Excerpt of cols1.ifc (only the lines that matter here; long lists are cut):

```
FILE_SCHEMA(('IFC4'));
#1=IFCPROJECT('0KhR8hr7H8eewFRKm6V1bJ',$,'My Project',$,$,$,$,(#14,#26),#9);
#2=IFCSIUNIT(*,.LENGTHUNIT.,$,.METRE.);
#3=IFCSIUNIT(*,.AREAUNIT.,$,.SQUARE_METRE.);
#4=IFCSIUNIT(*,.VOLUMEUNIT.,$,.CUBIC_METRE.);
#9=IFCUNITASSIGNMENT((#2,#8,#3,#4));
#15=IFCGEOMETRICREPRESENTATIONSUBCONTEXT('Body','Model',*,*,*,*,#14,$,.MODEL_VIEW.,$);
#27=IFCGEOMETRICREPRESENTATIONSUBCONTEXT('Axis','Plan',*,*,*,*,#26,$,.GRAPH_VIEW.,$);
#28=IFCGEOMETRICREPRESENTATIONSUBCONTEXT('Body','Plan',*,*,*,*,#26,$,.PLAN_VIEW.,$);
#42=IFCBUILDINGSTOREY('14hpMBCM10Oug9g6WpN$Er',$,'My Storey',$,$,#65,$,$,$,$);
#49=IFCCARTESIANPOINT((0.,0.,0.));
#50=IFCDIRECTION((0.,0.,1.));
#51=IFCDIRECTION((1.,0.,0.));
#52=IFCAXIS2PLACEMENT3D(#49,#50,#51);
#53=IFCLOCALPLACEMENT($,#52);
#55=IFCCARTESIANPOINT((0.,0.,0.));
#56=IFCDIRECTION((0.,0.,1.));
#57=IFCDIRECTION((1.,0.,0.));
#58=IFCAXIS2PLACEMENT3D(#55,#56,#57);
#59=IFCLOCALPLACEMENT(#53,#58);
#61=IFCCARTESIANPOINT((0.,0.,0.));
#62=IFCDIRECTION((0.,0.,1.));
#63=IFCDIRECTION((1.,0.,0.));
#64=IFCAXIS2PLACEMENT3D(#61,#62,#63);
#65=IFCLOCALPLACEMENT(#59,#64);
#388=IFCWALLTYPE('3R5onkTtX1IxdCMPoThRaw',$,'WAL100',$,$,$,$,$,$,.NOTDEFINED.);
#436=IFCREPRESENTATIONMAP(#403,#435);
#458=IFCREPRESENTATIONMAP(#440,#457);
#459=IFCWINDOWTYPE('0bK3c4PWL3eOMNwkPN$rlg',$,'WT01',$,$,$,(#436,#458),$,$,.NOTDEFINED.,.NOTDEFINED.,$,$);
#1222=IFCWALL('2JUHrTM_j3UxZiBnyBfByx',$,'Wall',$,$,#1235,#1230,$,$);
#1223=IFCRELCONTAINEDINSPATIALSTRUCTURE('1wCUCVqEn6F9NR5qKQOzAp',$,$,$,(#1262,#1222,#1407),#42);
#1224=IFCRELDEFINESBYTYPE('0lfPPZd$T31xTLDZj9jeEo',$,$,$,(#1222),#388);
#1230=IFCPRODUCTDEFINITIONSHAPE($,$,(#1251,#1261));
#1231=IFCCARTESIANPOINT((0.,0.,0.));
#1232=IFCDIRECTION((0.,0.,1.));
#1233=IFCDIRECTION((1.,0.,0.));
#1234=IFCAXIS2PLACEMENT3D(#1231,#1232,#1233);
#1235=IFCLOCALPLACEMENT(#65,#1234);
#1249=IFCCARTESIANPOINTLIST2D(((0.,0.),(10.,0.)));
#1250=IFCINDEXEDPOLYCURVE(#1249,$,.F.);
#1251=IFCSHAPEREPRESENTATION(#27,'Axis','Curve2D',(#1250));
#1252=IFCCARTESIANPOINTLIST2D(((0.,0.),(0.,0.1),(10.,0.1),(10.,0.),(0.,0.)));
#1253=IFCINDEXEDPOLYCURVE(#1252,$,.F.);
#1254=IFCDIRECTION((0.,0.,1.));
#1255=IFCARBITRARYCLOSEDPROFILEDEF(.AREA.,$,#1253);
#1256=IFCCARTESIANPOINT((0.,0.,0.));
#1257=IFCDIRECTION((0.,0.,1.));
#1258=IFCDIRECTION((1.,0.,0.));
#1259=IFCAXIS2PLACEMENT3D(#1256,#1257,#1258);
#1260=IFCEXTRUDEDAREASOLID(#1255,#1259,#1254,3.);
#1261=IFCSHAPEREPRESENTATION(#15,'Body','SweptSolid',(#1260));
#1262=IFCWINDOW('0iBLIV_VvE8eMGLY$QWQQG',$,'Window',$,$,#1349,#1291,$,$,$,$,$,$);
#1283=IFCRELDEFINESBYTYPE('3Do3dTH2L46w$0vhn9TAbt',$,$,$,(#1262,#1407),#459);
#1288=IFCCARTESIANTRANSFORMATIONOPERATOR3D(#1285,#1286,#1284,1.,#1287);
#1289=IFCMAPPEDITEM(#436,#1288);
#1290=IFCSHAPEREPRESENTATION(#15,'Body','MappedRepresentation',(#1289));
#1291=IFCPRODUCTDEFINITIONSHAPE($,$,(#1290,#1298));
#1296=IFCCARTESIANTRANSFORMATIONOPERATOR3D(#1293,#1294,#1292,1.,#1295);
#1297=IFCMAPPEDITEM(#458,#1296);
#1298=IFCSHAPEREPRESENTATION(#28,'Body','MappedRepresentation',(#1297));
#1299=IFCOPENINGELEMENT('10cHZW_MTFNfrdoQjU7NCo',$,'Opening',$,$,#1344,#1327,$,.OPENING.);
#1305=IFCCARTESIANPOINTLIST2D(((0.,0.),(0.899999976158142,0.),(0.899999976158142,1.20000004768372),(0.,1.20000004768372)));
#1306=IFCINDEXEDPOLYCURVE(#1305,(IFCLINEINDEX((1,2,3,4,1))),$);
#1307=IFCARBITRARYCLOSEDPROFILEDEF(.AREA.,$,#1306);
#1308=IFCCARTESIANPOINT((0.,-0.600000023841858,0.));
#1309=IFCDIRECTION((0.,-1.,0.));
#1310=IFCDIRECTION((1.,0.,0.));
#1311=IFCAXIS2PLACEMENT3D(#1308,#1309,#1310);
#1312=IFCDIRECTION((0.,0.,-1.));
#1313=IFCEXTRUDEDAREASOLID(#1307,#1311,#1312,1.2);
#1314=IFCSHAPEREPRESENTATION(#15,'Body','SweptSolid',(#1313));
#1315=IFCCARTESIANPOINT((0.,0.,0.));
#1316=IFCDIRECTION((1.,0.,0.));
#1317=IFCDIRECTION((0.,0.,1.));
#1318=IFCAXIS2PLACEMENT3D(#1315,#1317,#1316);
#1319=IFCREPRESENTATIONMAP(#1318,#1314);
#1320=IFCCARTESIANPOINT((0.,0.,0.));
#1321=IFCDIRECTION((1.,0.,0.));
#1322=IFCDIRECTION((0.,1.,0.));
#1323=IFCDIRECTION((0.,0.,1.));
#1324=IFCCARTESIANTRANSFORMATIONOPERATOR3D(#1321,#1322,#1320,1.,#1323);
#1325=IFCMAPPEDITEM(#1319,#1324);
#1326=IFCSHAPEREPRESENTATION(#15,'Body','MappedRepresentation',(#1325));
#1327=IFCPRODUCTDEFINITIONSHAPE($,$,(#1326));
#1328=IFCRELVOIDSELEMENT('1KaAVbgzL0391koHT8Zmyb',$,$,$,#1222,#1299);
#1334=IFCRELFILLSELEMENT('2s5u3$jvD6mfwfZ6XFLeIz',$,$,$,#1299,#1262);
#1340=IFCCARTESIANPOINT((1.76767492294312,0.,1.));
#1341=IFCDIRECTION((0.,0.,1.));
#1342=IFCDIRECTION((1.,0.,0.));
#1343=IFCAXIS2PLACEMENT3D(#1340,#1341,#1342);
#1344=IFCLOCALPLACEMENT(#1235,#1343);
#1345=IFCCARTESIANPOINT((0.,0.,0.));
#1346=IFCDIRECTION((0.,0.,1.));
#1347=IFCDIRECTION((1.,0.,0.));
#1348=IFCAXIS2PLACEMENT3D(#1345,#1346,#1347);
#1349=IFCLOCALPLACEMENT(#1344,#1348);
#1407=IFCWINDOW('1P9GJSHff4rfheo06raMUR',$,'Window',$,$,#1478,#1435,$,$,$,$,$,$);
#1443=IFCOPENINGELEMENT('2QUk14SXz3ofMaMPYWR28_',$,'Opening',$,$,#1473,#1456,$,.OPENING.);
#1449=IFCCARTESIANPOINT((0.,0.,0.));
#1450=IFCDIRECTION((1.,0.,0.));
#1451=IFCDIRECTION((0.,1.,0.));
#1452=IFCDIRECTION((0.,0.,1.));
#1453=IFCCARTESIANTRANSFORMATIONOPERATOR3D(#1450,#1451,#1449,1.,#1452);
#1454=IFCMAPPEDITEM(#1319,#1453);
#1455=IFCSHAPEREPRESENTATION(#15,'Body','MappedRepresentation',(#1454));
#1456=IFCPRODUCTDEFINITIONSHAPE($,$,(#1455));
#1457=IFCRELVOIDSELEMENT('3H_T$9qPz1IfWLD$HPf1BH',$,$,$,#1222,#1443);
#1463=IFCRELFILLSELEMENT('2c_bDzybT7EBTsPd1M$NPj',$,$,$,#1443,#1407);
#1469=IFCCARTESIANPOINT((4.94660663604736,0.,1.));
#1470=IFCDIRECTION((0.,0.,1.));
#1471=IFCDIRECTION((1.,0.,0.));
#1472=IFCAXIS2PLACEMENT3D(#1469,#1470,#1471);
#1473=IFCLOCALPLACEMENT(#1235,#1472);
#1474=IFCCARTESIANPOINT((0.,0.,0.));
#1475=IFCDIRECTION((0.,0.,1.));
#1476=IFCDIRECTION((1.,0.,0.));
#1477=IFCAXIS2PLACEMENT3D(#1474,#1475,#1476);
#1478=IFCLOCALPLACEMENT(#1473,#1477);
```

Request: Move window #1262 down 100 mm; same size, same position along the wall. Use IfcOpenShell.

```python
import numpy as np
import ifcopenshell
import ifcopenshell.api.geometry
import ifcopenshell.util.placement
import ifcopenshell.util.unit

model = ifcopenshell.open("cols1.ifc")
unit_scale = ifcopenshell.util.unit.calculate_unit_scale(model)

window = model.by_id(1262)
opening = window.FillsVoids[0].RelatingOpeningElement
dz = -0.1

shift = np.array([0.0, 0.0, dz])
# The window is placed relative to its opening, so it follows when the opening moves.
matrix = ifcopenshell.util.placement.get_local_placement(opening.ObjectPlacement)
matrix[:3, 3] += shift
ifcopenshell.api.geometry.edit_object_placement(
    model, product=opening, matrix=matrix, is_si=False, should_transform_children=True
)

print(f"moved by {dz * unit_scale:+.3f} m")

model.write("cols1_v2.ifc")
```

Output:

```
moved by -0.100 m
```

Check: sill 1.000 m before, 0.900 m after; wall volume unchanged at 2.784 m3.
